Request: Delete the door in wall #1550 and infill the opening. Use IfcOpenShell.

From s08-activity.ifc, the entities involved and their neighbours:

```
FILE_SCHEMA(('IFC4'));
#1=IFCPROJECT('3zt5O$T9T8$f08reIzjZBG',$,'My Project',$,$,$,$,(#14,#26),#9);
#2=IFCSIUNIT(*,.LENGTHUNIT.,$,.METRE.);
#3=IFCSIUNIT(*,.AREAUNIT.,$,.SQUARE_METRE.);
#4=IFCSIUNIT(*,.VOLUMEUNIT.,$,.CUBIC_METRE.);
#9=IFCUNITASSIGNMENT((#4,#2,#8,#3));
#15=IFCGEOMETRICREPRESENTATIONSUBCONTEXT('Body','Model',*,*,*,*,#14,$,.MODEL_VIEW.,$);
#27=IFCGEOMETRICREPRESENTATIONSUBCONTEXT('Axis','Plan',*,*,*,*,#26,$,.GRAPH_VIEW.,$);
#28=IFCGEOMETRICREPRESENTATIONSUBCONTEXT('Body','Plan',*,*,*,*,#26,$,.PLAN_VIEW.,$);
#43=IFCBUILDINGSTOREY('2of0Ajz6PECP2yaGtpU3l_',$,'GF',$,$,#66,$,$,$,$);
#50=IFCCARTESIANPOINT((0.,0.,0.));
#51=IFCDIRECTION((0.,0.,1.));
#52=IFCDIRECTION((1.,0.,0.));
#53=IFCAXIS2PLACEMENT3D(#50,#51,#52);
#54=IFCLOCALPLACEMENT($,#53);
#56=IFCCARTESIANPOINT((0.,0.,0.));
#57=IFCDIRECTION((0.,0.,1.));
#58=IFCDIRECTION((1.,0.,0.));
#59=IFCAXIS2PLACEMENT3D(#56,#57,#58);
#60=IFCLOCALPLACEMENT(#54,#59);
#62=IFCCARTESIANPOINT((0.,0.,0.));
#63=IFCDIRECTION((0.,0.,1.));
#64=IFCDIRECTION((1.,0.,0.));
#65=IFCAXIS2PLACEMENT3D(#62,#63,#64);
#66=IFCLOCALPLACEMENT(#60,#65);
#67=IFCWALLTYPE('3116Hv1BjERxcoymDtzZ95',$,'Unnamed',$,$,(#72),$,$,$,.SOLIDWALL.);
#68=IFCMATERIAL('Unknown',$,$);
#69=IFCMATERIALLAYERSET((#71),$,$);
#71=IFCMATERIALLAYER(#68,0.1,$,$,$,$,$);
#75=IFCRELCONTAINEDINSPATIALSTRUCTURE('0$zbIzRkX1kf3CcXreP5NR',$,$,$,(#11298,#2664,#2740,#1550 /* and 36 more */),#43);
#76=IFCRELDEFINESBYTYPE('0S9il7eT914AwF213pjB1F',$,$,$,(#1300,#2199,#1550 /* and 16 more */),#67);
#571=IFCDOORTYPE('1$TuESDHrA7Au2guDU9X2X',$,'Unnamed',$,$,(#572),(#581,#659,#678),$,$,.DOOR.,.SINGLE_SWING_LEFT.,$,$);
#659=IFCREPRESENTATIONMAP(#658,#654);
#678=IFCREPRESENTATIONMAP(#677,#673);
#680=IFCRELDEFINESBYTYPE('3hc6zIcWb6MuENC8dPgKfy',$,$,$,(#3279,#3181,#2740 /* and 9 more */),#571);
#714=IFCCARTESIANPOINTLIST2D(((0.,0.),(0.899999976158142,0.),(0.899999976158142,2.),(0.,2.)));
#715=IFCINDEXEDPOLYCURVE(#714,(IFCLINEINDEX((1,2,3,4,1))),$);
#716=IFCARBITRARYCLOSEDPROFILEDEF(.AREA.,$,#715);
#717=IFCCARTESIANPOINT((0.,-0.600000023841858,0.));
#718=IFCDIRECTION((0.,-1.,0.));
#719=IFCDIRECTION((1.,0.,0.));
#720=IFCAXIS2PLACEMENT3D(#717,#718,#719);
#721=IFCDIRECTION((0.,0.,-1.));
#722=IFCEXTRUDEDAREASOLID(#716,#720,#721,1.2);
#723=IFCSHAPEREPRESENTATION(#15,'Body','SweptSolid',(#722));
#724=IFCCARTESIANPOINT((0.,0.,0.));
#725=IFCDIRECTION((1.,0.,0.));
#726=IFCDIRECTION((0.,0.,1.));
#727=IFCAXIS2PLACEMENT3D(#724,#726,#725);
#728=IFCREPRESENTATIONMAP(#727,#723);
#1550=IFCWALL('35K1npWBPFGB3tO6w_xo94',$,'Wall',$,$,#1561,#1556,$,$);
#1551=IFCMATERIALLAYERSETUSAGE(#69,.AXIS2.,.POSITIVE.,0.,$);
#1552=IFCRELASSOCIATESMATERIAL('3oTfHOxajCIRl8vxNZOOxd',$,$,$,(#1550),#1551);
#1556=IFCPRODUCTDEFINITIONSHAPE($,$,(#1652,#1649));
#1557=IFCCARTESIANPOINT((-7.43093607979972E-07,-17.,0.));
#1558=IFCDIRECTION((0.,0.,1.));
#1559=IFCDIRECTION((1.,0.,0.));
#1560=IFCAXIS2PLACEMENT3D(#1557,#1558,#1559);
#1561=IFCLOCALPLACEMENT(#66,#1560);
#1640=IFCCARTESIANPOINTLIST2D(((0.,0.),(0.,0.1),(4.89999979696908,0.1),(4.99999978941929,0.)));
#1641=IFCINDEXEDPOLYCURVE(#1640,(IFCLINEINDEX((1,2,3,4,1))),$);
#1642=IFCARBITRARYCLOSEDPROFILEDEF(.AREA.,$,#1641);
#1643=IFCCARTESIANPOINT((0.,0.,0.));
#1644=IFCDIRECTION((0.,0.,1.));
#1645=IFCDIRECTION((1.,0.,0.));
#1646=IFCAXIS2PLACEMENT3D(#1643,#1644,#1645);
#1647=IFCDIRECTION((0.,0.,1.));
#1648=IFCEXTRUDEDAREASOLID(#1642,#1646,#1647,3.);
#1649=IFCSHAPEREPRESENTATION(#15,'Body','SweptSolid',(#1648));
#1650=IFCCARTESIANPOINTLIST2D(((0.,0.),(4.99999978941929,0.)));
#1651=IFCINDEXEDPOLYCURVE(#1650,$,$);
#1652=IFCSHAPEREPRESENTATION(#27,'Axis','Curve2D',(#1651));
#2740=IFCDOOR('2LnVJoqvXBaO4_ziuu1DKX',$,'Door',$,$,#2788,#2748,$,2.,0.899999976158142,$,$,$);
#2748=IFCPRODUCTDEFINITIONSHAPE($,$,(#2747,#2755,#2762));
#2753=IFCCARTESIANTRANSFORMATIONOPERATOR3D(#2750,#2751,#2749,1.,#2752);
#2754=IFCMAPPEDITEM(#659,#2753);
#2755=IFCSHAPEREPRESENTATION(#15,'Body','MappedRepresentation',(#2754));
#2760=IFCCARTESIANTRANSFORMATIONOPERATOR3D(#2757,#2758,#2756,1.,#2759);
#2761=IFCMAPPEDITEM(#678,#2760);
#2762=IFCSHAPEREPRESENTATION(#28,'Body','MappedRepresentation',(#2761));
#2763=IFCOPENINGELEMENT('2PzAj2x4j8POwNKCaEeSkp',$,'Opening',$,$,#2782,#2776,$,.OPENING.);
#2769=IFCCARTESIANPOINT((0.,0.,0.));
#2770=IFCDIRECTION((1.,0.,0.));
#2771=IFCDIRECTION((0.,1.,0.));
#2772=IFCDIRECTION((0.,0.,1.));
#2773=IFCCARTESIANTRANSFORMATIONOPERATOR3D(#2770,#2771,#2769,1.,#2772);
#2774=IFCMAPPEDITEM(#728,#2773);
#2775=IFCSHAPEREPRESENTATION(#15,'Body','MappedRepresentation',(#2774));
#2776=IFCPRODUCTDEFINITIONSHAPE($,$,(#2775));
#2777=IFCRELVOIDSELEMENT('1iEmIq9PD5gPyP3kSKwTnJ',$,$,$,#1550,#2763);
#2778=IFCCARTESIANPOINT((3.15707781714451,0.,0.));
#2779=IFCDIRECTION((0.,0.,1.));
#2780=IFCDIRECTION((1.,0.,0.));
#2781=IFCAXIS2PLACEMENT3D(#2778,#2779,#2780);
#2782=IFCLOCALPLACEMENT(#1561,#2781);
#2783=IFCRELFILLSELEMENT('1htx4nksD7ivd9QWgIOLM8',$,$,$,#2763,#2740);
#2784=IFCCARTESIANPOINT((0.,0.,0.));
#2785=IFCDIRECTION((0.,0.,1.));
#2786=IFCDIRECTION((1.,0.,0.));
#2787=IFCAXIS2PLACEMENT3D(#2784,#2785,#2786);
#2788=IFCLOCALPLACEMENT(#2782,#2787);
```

```python
import ifcopenshell
import ifcopenshell.api.feature
import ifcopenshell.api.root
import ifcopenshell.geom
import ifcopenshell.util.shape

model = ifcopenshell.open("s08-activity.ifc")
settings = ifcopenshell.geom.settings()


def volume(element):
    """Net volume in cubic metres, openings subtracted."""
    shape = ifcopenshell.geom.create_shape(settings, element)
    return ifcopenshell.util.shape.get_volume(shape.geometry)


door = model.by_id(2740)
opening = door.FillsVoids[0].RelatingOpeningElement
wall = opening.VoidsElements[0].RelatingBuildingElement
before = volume(wall)

ifcopenshell.api.root.remove_product(model, product=door)
ifcopenshell.api.feature.remove_feature(model, feature=opening)

after = volume(wall)

print(f"wall volume {before:.3f} -> {after:.3f} m3")

model.write("s08-activity_edited.ifc")
```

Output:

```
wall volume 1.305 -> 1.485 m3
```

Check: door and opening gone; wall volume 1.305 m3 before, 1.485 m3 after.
